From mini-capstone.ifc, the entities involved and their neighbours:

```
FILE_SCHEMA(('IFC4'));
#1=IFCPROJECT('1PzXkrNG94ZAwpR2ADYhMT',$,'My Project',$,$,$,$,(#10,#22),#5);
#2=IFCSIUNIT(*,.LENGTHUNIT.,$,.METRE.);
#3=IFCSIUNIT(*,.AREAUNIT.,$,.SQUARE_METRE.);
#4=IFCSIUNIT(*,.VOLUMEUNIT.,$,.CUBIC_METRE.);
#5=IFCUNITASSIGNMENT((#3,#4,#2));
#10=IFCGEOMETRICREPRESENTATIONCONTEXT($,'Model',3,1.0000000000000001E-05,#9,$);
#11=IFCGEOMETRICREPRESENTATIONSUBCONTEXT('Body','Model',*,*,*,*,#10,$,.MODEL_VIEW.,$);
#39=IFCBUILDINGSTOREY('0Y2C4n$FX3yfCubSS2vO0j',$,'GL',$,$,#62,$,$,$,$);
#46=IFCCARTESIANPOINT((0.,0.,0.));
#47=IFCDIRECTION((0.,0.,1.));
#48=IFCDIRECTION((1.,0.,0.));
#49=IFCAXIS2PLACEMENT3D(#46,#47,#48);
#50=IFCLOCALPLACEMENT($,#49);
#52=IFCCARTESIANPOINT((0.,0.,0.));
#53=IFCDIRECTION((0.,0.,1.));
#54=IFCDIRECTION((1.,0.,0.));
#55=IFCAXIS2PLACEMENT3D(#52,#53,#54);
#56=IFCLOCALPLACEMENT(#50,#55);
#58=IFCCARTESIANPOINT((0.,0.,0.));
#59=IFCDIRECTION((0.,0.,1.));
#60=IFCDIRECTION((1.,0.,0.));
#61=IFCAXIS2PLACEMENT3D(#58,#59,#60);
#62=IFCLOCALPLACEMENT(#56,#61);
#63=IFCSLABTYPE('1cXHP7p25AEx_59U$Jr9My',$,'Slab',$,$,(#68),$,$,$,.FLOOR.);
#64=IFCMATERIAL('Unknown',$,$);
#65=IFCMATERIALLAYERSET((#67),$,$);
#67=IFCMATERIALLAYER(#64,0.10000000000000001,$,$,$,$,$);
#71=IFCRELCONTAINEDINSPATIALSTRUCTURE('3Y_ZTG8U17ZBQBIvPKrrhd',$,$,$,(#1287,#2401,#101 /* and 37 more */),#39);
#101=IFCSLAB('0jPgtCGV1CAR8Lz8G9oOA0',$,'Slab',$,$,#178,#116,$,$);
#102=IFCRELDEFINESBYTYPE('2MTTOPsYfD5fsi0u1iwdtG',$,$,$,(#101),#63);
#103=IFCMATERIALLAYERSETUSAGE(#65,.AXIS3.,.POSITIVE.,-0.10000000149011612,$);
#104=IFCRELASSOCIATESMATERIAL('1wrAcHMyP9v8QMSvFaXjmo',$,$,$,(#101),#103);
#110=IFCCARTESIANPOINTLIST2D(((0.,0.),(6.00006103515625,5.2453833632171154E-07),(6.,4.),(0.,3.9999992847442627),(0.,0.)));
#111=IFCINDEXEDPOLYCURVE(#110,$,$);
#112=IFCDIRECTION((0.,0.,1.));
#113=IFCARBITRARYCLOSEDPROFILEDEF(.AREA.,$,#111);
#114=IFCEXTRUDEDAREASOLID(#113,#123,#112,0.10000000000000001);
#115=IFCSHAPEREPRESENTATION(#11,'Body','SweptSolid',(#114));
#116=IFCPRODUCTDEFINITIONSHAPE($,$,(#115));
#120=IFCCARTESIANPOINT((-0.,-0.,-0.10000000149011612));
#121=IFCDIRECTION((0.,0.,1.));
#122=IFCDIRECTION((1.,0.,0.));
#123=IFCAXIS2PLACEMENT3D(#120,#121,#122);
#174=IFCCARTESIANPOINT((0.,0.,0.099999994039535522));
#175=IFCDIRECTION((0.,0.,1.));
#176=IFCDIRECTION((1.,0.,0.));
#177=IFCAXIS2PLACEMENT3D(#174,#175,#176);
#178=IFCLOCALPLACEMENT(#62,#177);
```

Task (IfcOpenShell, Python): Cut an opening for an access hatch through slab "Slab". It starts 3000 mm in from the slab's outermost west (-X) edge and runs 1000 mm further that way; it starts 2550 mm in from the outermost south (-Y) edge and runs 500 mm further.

```python
import numpy as np
import ifcopenshell
import ifcopenshell.api.feature
import ifcopenshell.api.geometry
import ifcopenshell.api.root
import ifcopenshell.geom
import ifcopenshell.util.placement
import ifcopenshell.util.representation
import ifcopenshell.util.shape
import ifcopenshell.util.unit

model = ifcopenshell.open("mini-capstone.ifc")
unit_scale = ifcopenshell.util.unit.calculate_unit_scale(model)
settings = ifcopenshell.geom.settings()


def volume(element):
    """Net volume in cubic metres, openings subtracted."""
    shape = ifcopenshell.geom.create_shape(settings, element)
    return ifcopenshell.util.shape.get_volume(shape.geometry)


slab = model.by_guid("0jPgtCGV1CAR8Lz8G9oOA0")
before = volume(slab)

# Extent in the slab's own axes, in metres. The edges named are its -X and -Y sides.
slab_shape = ifcopenshell.geom.create_shape(settings, slab)
vertices = ifcopenshell.util.shape.get_vertices(slab_shape.geometry)
x_min, y_min, bottom = vertices.min(axis=0)
top = vertices[:, 2].max()

opening = ifcopenshell.api.root.create_entity(model, ifc_class="IfcOpeningElement", name="Access hatch opening", predefined_type="OPENING")
context = ifcopenshell.util.representation.get_context(model, "Model", "Body", "MODEL_VIEW")
width, depth = 1, 0.5
outline = [(0.0, 0.0), (width, 0.0), (width, depth), (0.0, depth), (0.0, 0.0)]
# Overshoot both faces by 50 mm so the cut is clean.
shape = ifcopenshell.api.geometry.add_slab_representation(
    model, context=context, depth=top - bottom + 0.1, polyline=outline
)
ifcopenshell.api.geometry.assign_representation(model, product=opening, representation=shape)

matrix = ifcopenshell.util.placement.get_local_placement(slab.ObjectPlacement)
matrix[:, 3] = matrix @ np.append(np.array([x_min + 3, y_min + 2.55, bottom - 0.05]) / unit_scale, 1.0)
ifcopenshell.api.geometry.edit_object_placement(model, product=opening, matrix=matrix, is_si=False)
ifcopenshell.api.feature.add_feature(model, feature=opening, element=slab)

after = volume(slab)

print(f"slab volume {before:.3f} -> {after:.3f} m3")

model.write("mini-capstone_updated.ifc")
```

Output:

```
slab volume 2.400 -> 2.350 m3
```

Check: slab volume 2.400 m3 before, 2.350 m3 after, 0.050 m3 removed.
